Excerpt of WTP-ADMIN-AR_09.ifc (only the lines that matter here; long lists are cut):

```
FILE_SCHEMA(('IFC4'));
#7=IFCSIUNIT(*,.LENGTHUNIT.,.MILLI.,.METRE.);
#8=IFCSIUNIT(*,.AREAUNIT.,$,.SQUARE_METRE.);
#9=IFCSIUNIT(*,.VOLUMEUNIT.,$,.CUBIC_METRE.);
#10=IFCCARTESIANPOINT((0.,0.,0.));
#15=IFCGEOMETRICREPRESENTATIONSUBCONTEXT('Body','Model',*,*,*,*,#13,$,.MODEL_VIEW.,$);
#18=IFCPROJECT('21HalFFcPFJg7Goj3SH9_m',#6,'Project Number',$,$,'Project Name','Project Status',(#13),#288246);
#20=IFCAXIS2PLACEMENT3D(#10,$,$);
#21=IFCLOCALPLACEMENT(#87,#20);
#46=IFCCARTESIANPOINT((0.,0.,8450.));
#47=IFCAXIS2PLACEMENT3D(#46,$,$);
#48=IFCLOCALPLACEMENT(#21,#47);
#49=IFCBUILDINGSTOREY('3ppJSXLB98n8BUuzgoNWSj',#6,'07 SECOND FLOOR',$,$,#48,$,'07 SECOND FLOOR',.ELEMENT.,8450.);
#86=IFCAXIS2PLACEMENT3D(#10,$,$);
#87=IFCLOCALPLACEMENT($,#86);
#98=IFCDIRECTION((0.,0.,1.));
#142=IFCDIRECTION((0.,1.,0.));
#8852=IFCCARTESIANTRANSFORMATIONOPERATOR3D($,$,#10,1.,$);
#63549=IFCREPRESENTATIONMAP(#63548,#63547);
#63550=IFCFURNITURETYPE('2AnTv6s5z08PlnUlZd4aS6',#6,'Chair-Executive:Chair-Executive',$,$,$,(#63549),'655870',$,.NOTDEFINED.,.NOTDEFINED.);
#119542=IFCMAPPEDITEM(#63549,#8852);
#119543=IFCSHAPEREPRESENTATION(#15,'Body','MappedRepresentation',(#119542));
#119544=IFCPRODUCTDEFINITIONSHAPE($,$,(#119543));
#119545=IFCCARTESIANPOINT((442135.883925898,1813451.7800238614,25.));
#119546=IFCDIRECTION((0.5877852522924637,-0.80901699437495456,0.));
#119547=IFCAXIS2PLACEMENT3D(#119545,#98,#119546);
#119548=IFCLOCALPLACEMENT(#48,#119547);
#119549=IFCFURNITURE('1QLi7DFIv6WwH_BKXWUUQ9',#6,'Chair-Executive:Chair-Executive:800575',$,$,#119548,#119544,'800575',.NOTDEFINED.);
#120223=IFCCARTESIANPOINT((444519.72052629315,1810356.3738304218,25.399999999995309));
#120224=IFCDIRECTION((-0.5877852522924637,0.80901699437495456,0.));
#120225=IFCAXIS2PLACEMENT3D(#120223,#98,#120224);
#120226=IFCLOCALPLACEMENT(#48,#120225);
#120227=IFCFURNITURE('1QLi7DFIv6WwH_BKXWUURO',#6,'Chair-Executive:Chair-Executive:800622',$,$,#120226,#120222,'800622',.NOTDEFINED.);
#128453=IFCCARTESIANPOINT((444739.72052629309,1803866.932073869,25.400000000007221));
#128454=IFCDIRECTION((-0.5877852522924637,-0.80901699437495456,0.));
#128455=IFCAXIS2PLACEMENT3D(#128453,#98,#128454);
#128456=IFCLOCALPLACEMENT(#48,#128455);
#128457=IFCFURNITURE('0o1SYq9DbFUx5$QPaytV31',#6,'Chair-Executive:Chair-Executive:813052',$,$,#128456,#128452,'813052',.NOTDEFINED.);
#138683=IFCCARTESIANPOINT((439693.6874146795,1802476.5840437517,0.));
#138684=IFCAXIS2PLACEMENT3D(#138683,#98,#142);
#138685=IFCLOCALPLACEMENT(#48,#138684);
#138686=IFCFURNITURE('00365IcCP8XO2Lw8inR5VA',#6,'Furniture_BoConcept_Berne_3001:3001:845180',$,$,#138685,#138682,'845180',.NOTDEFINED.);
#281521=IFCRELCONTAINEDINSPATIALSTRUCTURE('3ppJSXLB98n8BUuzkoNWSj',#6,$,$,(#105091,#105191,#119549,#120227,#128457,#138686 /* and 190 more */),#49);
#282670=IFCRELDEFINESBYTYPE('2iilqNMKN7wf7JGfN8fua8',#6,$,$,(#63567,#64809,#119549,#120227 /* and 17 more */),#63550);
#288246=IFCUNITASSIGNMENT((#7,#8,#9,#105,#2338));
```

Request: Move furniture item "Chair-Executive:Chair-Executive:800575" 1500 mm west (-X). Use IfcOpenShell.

```python
import ifcopenshell
import ifcopenshell.api.geometry
import ifcopenshell.util.placement
import ifcopenshell.util.unit

model = ifcopenshell.open("WTP-ADMIN-AR_09.ifc")
unit_scale = ifcopenshell.util.unit.calculate_unit_scale(model)

item = model.by_id(119549)
matrix = ifcopenshell.util.placement.get_local_placement(item.ObjectPlacement)
matrix[0, 3] -= 1.5 / unit_scale
ifcopenshell.api.geometry.edit_object_placement(model, product=item, matrix=matrix, is_si=False)

print(ifcopenshell.util.placement.get_local_placement(item.ObjectPlacement).round(3) + 0.0)

model.write("WTP-ADMIN-AR_09_rev.ifc")
```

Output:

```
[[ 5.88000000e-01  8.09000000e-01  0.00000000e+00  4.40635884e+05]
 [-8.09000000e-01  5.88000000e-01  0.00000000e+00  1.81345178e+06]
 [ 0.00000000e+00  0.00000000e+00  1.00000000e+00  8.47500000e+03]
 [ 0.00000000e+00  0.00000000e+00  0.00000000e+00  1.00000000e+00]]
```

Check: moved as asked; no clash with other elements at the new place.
